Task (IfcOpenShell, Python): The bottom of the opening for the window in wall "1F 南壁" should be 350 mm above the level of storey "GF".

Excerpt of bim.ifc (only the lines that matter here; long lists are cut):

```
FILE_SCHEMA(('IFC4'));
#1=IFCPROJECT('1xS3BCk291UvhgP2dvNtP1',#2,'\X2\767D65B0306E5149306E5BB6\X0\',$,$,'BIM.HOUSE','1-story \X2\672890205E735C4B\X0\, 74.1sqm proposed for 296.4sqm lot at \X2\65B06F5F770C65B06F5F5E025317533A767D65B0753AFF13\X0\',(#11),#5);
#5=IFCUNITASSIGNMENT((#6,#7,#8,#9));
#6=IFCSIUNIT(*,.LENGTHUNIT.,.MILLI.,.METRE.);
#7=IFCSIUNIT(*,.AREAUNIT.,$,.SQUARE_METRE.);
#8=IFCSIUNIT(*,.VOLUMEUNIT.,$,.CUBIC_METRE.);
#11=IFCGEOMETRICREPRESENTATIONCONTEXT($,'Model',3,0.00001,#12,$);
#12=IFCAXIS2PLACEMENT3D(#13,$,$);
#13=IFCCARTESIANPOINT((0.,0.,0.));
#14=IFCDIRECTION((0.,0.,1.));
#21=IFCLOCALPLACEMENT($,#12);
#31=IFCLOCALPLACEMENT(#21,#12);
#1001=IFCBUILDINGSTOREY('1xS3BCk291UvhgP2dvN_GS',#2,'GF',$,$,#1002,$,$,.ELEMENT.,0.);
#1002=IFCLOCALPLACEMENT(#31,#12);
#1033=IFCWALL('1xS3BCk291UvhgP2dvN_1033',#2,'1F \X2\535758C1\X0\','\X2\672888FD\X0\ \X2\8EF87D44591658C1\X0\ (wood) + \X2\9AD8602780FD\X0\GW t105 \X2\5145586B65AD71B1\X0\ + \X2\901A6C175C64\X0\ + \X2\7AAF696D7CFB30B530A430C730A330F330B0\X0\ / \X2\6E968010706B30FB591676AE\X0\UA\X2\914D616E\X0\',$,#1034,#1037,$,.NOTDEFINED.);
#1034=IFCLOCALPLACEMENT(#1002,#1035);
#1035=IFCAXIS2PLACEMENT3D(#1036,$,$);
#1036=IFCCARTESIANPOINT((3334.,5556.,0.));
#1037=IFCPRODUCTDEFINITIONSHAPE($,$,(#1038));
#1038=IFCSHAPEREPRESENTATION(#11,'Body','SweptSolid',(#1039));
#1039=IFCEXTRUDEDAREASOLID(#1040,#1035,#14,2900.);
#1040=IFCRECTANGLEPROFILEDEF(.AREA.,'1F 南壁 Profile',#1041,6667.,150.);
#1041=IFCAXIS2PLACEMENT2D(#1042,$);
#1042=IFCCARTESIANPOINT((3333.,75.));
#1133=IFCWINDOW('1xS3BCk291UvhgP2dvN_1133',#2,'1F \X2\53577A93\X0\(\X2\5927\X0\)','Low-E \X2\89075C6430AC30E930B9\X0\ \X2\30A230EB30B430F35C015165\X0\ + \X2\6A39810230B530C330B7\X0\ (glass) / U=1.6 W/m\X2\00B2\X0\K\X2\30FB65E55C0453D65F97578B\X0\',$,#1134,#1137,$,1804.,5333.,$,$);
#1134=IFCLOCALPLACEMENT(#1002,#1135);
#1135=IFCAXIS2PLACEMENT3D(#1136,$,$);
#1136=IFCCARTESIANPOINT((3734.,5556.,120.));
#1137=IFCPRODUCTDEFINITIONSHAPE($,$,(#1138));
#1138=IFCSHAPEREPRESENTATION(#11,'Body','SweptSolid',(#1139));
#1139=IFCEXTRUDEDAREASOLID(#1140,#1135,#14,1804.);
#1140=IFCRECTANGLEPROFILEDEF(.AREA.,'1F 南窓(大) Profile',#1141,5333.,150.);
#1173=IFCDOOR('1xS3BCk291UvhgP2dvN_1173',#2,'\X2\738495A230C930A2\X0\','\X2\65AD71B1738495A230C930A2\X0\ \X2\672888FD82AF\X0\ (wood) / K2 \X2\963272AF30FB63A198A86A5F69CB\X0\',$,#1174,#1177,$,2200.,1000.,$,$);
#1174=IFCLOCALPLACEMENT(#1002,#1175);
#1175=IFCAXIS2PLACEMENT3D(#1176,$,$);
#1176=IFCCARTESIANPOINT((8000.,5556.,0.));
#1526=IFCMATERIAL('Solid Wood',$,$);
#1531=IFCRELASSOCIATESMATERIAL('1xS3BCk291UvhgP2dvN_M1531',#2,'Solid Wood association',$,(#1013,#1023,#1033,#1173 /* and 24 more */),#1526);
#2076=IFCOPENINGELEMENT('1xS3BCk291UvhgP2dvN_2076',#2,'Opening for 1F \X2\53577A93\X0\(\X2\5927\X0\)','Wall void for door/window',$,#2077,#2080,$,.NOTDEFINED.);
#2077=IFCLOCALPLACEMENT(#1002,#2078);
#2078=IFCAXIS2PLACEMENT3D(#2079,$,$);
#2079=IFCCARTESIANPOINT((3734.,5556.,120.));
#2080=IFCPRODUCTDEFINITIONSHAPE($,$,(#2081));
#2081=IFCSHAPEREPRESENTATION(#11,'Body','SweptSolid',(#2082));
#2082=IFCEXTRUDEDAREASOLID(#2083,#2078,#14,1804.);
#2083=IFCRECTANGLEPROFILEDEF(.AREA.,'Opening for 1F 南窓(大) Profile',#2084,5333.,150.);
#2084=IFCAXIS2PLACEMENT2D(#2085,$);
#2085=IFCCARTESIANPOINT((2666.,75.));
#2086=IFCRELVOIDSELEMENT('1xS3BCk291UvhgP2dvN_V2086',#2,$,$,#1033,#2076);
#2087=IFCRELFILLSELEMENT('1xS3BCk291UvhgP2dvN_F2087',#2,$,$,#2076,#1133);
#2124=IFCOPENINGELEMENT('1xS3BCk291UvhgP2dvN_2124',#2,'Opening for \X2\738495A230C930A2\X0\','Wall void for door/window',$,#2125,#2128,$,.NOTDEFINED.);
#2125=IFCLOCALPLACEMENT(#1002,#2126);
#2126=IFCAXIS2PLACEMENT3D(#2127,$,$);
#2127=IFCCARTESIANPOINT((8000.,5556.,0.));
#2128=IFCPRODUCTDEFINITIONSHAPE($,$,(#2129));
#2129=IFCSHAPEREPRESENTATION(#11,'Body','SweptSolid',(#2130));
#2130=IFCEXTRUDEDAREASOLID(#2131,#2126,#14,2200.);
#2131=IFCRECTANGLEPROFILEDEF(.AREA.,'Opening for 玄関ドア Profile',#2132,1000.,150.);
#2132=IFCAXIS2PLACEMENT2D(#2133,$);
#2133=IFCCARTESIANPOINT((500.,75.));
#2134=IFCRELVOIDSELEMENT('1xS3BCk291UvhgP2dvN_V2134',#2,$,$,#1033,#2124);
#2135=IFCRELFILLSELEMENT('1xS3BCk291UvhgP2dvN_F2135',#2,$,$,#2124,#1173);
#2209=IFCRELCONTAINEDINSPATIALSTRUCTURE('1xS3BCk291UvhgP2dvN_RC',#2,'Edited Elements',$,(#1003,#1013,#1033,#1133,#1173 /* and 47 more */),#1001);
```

```python
import numpy as np
import ifcopenshell
import ifcopenshell.api.geometry
import ifcopenshell.geom
import ifcopenshell.util.element
import ifcopenshell.util.placement
import ifcopenshell.util.shape
import ifcopenshell.util.unit

model = ifcopenshell.open("bim.ifc")
unit_scale = ifcopenshell.util.unit.calculate_unit_scale(model)

window = model.by_guid("1xS3BCk291UvhgP2dvN_1133")
opening = window.FillsVoids[0].RelatingOpeningElement
storey = ifcopenshell.util.element.get_container(window, ifc_class="IfcBuildingStorey")
level = ifcopenshell.util.placement.get_local_placement(storey.ObjectPlacement)[2, 3]

# The opening's origin need not be at the sill, so measure its lowest point.
shape = ifcopenshell.geom.create_shape(ifcopenshell.geom.settings(), opening)
bottom = ifcopenshell.util.shape.get_shape_bottom_elevation(shape, shape.geometry) / unit_scale
dz = level + 0.35 / unit_scale - bottom

shift = np.array([0.0, 0.0, dz])
# The window is not placed relative to its opening, so move both.
for product in (opening, window):
    matrix = ifcopenshell.util.placement.get_local_placement(product.ObjectPlacement)
    matrix[:3, 3] += shift
    ifcopenshell.api.geometry.edit_object_placement(model, product=product, matrix=matrix, is_si=False)

print(f"moved by {dz * unit_scale:+.3f} m")

model.write("bim_v2.ifc")
```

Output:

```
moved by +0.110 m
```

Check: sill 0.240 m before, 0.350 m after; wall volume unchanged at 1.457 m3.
